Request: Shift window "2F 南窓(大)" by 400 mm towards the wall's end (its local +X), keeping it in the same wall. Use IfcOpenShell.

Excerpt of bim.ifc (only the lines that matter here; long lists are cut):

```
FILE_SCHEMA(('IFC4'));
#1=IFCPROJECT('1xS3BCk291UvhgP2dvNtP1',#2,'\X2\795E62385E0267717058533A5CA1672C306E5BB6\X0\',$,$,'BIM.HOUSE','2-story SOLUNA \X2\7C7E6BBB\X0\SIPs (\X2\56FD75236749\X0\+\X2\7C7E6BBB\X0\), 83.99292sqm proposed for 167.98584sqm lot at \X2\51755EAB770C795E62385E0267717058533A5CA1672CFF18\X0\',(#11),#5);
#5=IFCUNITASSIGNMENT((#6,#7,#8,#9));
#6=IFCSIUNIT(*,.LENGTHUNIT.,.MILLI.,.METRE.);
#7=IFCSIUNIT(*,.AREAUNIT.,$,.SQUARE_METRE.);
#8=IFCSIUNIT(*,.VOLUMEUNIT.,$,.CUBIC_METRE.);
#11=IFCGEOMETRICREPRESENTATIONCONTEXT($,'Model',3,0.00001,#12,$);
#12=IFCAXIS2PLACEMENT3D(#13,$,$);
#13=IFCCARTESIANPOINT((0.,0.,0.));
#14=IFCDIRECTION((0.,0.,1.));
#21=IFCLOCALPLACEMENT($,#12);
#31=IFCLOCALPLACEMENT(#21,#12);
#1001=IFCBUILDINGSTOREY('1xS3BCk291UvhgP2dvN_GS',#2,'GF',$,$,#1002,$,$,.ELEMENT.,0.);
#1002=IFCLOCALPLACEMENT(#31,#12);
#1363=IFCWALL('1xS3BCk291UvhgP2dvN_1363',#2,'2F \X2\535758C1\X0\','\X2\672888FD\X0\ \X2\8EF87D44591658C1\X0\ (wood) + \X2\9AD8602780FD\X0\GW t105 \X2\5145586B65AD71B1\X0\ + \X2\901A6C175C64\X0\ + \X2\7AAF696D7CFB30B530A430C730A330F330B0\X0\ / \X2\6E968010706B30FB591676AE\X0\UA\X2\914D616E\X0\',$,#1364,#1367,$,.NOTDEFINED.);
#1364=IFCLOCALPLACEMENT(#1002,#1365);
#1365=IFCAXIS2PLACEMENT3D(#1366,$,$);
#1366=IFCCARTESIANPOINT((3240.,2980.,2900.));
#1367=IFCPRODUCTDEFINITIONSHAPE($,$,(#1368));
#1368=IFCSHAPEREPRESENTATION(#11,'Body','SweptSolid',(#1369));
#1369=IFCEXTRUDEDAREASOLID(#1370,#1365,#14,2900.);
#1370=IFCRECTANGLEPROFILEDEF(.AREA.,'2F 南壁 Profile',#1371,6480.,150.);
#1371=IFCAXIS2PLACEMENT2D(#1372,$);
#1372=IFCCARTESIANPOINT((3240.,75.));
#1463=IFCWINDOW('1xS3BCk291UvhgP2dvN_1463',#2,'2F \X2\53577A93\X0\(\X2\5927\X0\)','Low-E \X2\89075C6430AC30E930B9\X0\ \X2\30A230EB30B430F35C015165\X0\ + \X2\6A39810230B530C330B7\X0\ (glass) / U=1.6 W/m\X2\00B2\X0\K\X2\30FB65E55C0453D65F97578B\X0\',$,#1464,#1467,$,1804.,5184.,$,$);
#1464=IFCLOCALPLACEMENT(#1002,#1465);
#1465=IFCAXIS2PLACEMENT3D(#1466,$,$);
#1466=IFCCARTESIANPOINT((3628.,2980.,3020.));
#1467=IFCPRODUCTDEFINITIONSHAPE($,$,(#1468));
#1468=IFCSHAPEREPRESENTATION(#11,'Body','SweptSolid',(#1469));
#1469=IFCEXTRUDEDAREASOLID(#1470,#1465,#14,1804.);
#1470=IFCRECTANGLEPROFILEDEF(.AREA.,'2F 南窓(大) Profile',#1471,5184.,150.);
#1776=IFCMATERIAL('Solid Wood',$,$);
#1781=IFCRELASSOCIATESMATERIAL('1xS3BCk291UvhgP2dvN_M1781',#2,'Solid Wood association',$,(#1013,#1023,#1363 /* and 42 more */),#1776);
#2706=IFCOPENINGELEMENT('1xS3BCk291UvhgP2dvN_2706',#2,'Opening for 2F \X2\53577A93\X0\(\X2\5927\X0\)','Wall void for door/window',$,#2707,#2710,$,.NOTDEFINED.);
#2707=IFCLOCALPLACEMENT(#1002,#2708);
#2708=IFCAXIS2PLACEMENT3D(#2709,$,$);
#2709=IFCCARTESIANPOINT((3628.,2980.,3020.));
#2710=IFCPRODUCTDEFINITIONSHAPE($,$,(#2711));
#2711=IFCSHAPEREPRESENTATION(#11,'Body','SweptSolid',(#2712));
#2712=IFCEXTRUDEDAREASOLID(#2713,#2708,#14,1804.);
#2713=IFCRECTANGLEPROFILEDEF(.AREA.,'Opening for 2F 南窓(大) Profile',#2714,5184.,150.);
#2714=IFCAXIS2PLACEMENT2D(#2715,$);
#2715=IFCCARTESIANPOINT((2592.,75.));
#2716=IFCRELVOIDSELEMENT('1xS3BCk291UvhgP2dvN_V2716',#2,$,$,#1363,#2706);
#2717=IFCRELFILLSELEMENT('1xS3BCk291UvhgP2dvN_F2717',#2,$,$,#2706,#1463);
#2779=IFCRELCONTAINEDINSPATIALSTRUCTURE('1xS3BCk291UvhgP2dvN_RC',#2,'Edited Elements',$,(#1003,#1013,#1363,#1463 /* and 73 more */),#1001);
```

```python
import ifcopenshell
import ifcopenshell.api.geometry
import ifcopenshell.util.placement
import ifcopenshell.util.unit

model = ifcopenshell.open("bim.ifc")
unit_scale = ifcopenshell.util.unit.calculate_unit_scale(model)

window = model.by_guid("1xS3BCk291UvhgP2dvN_1463")
opening = window.FillsVoids[0].RelatingOpeningElement
wall = opening.VoidsElements[0].RelatingBuildingElement

wall_matrix = ifcopenshell.util.placement.get_local_placement(wall.ObjectPlacement)
shift = wall_matrix[:3, 0] * 0.4 / unit_scale
before = ifcopenshell.util.placement.get_local_placement(window.ObjectPlacement)[:3, 3].copy()

# The window is not placed relative to its opening, so move both.
for product in (opening, window):
    matrix = ifcopenshell.util.placement.get_local_placement(product.ObjectPlacement)
    matrix[:3, 3] += shift
    ifcopenshell.api.geometry.edit_object_placement(model, product=product, matrix=matrix, is_si=False)

after = ifcopenshell.util.placement.get_local_placement(window.ObjectPlacement)[:3, 3]
print("window moved by", (after - before).round(3) + 0.0)

model.write("bim_updated.ifc")
```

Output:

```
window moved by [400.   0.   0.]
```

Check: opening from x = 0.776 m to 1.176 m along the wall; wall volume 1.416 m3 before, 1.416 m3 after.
